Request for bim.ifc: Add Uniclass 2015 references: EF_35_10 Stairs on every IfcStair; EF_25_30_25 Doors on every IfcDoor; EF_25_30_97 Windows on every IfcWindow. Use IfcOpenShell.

First a look at what the model holds.

```python
import ifcopenshell

model = ifcopenshell.open("bim.ifc")
print(model.schema)
print("classifications:", [c.Name for c in model.by_type("IfcClassification")])
for ifc_class in ("IfcDoor", "IfcRoof", "IfcStair", "IfcWall", "IfcWindow"):
    print(ifc_class, len(model.by_type(ifc_class)))
```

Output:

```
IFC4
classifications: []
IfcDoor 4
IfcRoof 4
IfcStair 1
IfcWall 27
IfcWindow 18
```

```python
import ifcopenshell
import ifcopenshell.api.classification

model = ifcopenshell.open("bim.ifc")

system = ifcopenshell.api.classification.add_classification(model, classification="Uniclass 2015")

codes = {
    "IfcStair": ("EF_35_10", "Stairs"),
    "IfcDoor": ("EF_25_30_25", "Doors"),
    "IfcWindow": ("EF_25_30_97", "Windows"),
}
for ifc_class, (code, name) in codes.items():
    products = model.by_type(ifc_class)
    ifcopenshell.api.classification.add_reference(
        model, products=products, classification=system, identification=code, name=name
    )
    print(code, len(products))

model.write("bim_rev.ifc")
```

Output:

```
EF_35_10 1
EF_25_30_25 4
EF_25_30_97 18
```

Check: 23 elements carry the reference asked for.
